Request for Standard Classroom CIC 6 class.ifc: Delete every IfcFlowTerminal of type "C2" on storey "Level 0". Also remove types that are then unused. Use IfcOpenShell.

First a look at what the model holds.

```python
import ifcopenshell
import ifcopenshell.util.element

model = ifcopenshell.open("Standard Classroom CIC 6 class.ifc")
print(model.schema)
storey = next(s for s in model.by_type("IfcBuildingStorey") if s.Name == "Level 0")
terminals = [e for e in ifcopenshell.util.element.get_decomposition(storey) if e.is_a("IfcFlowTerminal")]
seen = {}
for e in terminals:
    element_type = ifcopenshell.util.element.get_type(e)
    name = element_type.Name if element_type not in (None, e) else None
    seen[name] = seen.get(name, 0) + 1
for name, count in sorted(seen.items(), key=str):
    print(count, "x", name)
```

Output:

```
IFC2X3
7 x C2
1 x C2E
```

```python
import ifcopenshell
import ifcopenshell.api.root
import ifcopenshell.util.element

model = ifcopenshell.open("Standard Classroom CIC 6 class.ifc")

storey = next(s for s in model.by_type("IfcBuildingStorey") if s.Name == "Level 0")
terminals = [e for e in ifcopenshell.util.element.get_decomposition(storey) if e.is_a("IfcFlowTerminal")]
targets = [e for e in terminals if (t := ifcopenshell.util.element.get_type(e)) not in (None, e) and t.Name == "C2"]
types = {ifcopenshell.util.element.get_type(e) for e in targets} - {None, *targets}

for e in targets:
    ifcopenshell.api.root.remove_product(model, product=e)
print(len(targets), "removed")

unused = [t for t in types if not ifcopenshell.util.element.get_types(t)]
for t in unused:
    ifcopenshell.api.root.remove_product(model, product=t)
print(len(unused), "unused types removed")

model.write("Standard Classroom CIC 6 class_updated.ifc")
```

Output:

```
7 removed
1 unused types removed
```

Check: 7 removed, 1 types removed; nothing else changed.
